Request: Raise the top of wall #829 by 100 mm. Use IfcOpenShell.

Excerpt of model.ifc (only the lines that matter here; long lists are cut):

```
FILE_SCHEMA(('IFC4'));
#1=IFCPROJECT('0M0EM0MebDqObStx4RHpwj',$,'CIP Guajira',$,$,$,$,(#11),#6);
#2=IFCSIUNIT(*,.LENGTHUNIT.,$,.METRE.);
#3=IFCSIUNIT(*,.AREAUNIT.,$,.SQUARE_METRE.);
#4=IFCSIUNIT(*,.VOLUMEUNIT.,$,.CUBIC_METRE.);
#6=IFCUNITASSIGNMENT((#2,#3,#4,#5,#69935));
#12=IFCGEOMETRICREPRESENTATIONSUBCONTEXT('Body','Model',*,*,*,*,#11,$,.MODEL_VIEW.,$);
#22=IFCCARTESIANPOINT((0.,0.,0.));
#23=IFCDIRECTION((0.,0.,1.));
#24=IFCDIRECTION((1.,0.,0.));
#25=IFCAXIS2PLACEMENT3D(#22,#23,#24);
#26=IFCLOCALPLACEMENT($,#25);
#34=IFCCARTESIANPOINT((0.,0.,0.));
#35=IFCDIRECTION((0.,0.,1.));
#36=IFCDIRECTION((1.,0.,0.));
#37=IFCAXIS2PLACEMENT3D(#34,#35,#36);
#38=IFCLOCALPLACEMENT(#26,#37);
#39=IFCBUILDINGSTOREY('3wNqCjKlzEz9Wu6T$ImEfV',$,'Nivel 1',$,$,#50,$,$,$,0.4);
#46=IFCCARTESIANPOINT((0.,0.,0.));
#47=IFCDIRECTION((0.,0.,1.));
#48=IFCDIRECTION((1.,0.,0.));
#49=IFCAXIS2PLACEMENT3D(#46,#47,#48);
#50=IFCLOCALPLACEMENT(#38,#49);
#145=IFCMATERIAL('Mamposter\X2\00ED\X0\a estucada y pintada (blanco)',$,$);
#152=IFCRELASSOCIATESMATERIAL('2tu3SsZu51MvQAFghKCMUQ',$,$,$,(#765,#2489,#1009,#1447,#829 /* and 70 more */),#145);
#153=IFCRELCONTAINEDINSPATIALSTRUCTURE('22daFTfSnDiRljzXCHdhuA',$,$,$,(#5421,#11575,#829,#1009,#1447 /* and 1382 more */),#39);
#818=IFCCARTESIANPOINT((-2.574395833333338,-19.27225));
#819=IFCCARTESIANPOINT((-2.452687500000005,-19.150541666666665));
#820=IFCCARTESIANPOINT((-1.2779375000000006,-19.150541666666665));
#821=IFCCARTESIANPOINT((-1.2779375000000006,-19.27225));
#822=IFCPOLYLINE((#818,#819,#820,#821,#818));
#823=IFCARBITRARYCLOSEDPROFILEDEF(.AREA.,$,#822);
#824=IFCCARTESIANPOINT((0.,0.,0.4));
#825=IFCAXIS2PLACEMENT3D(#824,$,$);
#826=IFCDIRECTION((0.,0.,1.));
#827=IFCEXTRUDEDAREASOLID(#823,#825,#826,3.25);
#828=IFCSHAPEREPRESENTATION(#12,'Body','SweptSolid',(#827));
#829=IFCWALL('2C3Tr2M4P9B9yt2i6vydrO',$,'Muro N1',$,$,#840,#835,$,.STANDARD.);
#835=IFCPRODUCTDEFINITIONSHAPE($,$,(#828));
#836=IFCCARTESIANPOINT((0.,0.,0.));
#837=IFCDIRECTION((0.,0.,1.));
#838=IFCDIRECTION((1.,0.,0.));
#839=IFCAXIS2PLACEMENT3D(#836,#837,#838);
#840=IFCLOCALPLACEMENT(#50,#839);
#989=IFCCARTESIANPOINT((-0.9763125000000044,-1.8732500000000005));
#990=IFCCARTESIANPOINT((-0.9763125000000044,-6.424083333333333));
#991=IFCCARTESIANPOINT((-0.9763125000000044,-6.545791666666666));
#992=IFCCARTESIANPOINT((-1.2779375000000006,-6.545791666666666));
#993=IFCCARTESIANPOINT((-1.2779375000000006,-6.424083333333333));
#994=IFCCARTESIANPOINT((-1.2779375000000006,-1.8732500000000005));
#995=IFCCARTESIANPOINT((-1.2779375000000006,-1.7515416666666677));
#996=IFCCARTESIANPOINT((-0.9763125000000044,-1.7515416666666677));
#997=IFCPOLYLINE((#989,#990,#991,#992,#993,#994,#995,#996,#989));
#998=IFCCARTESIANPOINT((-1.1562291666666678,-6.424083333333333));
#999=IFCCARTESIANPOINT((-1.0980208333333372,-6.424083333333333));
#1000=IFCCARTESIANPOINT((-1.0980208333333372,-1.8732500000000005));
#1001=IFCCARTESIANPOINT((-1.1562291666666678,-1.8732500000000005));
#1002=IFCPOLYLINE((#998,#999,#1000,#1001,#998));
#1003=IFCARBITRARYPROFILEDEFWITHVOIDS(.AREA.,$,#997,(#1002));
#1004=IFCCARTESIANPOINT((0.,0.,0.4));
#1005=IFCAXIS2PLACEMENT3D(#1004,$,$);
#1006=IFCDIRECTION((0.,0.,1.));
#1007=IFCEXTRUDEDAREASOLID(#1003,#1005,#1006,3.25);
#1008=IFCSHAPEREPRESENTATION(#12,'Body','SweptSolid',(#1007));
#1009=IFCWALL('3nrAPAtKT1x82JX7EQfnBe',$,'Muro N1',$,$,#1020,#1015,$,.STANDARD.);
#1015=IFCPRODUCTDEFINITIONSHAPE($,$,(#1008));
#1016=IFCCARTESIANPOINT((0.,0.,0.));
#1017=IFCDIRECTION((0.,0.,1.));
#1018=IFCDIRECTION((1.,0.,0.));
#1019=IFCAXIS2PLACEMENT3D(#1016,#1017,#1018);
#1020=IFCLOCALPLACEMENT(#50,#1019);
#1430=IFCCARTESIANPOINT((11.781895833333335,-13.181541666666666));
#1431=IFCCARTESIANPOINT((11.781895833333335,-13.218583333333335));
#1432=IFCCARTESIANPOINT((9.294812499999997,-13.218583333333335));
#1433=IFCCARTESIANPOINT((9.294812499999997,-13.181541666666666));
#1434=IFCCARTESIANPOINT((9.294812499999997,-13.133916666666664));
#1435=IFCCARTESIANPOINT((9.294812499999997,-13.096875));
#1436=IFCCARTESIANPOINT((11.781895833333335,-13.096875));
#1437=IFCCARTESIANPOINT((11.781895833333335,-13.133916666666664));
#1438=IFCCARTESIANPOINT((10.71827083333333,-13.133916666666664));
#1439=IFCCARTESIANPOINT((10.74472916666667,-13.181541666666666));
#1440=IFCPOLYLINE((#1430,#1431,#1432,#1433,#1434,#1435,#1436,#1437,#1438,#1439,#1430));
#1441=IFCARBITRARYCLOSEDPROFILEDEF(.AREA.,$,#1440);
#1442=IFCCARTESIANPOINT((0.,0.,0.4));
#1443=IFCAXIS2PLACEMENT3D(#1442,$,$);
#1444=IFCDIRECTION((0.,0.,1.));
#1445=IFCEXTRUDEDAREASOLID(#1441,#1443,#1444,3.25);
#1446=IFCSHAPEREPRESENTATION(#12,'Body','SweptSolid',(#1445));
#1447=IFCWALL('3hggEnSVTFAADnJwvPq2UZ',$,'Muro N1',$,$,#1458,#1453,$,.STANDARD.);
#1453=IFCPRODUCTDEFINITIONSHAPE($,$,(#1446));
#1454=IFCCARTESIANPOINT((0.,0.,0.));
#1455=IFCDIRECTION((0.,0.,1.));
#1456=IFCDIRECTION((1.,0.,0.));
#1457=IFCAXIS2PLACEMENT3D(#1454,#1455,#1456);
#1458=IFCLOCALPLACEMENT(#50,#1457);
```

```python
import ifcopenshell
import ifcopenshell.geom
import ifcopenshell.util.representation
import ifcopenshell.util.shape
import ifcopenshell.util.unit

model = ifcopenshell.open("model.ifc")
unit_scale = ifcopenshell.util.unit.calculate_unit_scale(model)
settings = ifcopenshell.geom.settings()


def volume(element):
    """Net volume in cubic metres, openings subtracted."""
    shape = ifcopenshell.geom.create_shape(settings, element)
    return ifcopenshell.util.shape.get_volume(shape.geometry)


wall = model.by_guid("2C3Tr2M4P9B9yt2i6vydrO")
before = volume(wall)

body = ifcopenshell.util.representation.get_representation(wall, "Model", "Body")
solid = body.Items[0]
old_height = solid.Depth
solid.Depth += 0.1 / unit_scale
after = volume(wall)

print(f"height {old_height:g} -> {solid.Depth:g}, volume {before:.3f} -> {after:.3f} m3")

model.write("model_rev.ifc")
```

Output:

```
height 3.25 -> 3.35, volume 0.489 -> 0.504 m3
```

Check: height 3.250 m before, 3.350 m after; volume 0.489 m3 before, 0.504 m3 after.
